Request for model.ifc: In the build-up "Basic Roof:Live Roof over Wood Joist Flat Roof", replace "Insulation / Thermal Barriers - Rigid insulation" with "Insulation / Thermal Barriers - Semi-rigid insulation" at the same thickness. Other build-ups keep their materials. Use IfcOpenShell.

First a look at what the model holds.

```python
import ifcopenshell
import ifcopenshell.util.element

model = ifcopenshell.open("model.ifc")
print(model.schema)
for layer_set in model.by_type("IfcMaterialLayerSet"):
    if layer_set.LayerSetName == "Basic Roof:Live Roof over Wood Joist Flat Roof":
        for layer in layer_set.MaterialLayers:
            print(layer.id(), layer.Material and layer.Material.Name, layer.LayerThickness, sep=" | ")
        print(len(ifcopenshell.util.element.get_elements_by_material(model, layer_set)), "elements and types use it")
print(sorted(m.Name for m in model.by_type("IfcMaterial") if m.Name)[:60])
```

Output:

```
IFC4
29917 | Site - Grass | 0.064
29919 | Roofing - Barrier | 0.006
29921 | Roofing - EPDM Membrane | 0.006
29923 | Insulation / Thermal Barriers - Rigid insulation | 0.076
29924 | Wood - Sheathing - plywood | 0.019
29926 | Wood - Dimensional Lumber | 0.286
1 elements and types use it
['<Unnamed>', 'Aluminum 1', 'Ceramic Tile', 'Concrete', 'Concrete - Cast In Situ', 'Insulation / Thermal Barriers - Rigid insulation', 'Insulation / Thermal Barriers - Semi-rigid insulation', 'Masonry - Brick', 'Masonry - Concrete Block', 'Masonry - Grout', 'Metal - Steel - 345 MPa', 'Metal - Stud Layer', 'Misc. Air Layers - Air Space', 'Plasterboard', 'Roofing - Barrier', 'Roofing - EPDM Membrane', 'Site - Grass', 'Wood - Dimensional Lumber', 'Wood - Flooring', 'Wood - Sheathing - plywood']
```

```python
import ifcopenshell
import ifcopenshell.api.material

model = ifcopenshell.open("model.ifc")

layer_set = next(s for s in model.by_type("IfcMaterialLayerSet") if s.LayerSetName == "Basic Roof:Live Roof over Wood Joist Flat Roof")
layer = next(l for l in layer_set.MaterialLayers if l.Material and l.Material.Name == "Insulation / Thermal Barriers - Rigid insulation")
material = next(m for m in model.by_type("IfcMaterial") if m.Name == "Insulation / Thermal Barriers - Semi-rigid insulation")

# Point this one layer at the other material; renaming the old one would change it everywhere.
ifcopenshell.api.material.edit_layer(model, layer=layer, attributes={}, material=material)

print([l.Material.Name if l.Material else None for l in layer_set.MaterialLayers])

model.write("model_edited.ifc")
```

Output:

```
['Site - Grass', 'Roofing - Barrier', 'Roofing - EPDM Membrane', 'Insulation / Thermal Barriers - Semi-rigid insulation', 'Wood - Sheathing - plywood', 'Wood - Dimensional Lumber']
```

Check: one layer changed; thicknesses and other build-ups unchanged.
